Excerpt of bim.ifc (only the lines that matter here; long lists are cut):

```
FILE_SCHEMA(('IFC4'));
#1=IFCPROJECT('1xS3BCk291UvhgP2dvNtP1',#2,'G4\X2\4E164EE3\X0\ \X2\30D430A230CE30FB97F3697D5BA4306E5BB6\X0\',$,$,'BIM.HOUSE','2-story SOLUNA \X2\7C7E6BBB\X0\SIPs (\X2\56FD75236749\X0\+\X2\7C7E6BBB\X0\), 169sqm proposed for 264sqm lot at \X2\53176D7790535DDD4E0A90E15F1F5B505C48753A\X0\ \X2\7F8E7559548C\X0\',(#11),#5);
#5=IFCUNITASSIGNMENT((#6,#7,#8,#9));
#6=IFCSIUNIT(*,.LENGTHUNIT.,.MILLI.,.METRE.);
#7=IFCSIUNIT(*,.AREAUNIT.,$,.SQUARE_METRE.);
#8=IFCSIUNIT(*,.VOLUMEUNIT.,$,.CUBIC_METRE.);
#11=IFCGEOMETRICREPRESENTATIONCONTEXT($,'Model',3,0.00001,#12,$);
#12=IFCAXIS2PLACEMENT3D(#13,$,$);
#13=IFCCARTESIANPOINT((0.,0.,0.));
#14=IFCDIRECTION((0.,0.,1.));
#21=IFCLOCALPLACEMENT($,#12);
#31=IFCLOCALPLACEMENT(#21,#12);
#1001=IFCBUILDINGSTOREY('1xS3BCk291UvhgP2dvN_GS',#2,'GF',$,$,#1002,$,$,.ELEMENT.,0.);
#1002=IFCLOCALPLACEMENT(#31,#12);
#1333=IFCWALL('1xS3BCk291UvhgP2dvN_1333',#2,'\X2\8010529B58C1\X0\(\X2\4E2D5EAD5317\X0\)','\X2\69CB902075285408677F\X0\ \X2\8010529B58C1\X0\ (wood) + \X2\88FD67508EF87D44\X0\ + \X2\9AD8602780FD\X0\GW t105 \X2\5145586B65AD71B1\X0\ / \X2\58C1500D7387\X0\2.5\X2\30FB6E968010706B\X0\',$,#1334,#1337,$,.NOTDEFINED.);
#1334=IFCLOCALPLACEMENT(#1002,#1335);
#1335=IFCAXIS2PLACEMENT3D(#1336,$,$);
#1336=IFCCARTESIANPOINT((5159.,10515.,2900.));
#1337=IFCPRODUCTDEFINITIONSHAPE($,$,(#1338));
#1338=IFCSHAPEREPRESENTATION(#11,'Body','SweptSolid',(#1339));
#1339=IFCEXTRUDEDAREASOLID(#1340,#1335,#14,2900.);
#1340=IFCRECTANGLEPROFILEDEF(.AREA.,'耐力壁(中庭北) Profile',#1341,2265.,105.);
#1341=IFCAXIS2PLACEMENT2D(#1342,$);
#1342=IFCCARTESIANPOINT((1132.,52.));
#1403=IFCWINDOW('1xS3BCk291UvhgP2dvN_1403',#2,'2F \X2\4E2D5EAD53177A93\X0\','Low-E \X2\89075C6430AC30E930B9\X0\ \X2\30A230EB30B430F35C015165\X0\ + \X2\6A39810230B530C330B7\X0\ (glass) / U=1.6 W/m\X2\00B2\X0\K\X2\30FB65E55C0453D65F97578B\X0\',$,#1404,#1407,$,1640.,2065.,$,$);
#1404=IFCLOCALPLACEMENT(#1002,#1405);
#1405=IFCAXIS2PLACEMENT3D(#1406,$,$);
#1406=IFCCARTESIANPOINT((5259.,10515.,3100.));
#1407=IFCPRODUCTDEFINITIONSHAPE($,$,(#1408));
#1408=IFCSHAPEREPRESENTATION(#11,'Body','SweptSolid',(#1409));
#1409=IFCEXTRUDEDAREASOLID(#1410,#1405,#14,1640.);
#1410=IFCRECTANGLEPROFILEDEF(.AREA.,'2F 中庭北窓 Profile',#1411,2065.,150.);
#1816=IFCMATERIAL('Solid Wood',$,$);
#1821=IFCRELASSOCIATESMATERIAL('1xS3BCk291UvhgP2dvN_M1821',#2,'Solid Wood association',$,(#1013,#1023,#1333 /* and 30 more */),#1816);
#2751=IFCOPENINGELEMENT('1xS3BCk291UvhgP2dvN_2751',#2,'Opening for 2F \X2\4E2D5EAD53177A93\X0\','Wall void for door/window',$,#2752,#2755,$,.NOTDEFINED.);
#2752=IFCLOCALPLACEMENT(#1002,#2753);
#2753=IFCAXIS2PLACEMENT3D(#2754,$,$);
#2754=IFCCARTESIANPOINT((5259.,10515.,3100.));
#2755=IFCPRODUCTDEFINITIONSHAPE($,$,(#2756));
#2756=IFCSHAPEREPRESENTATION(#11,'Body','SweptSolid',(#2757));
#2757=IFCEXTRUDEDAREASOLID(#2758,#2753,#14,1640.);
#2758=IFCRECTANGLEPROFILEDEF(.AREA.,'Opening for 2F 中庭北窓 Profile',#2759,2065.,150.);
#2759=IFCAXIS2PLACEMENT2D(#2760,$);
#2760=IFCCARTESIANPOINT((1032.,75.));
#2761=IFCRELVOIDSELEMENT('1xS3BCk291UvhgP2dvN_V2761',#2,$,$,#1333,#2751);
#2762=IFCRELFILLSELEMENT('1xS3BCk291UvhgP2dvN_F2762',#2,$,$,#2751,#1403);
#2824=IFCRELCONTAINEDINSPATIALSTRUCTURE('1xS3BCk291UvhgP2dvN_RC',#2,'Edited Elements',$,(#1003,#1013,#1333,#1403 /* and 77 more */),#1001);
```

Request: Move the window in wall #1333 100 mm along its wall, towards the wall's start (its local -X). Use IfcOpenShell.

```python
import ifcopenshell
import ifcopenshell.api.geometry
import ifcopenshell.util.placement
import ifcopenshell.util.unit

model = ifcopenshell.open("bim.ifc")
unit_scale = ifcopenshell.util.unit.calculate_unit_scale(model)

window = model.by_id(1403)
opening = window.FillsVoids[0].RelatingOpeningElement
wall = opening.VoidsElements[0].RelatingBuildingElement

wall_matrix = ifcopenshell.util.placement.get_local_placement(wall.ObjectPlacement)
shift = wall_matrix[:3, 0] * -0.1 / unit_scale
before = ifcopenshell.util.placement.get_local_placement(window.ObjectPlacement)[:3, 3].copy()

# The window is not placed relative to its opening, so move both.
for product in (opening, window):
    matrix = ifcopenshell.util.placement.get_local_placement(product.ObjectPlacement)
    matrix[:3, 3] += shift
    ifcopenshell.api.geometry.edit_object_placement(model, product=product, matrix=matrix, is_si=False)

after = ifcopenshell.util.placement.get_local_placement(window.ObjectPlacement)[:3, 3]
print("window moved by", (after - before).round(3) + 0.0)

model.write("bim_v2.ifc")
```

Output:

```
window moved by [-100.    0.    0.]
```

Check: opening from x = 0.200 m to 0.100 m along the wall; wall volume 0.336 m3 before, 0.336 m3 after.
